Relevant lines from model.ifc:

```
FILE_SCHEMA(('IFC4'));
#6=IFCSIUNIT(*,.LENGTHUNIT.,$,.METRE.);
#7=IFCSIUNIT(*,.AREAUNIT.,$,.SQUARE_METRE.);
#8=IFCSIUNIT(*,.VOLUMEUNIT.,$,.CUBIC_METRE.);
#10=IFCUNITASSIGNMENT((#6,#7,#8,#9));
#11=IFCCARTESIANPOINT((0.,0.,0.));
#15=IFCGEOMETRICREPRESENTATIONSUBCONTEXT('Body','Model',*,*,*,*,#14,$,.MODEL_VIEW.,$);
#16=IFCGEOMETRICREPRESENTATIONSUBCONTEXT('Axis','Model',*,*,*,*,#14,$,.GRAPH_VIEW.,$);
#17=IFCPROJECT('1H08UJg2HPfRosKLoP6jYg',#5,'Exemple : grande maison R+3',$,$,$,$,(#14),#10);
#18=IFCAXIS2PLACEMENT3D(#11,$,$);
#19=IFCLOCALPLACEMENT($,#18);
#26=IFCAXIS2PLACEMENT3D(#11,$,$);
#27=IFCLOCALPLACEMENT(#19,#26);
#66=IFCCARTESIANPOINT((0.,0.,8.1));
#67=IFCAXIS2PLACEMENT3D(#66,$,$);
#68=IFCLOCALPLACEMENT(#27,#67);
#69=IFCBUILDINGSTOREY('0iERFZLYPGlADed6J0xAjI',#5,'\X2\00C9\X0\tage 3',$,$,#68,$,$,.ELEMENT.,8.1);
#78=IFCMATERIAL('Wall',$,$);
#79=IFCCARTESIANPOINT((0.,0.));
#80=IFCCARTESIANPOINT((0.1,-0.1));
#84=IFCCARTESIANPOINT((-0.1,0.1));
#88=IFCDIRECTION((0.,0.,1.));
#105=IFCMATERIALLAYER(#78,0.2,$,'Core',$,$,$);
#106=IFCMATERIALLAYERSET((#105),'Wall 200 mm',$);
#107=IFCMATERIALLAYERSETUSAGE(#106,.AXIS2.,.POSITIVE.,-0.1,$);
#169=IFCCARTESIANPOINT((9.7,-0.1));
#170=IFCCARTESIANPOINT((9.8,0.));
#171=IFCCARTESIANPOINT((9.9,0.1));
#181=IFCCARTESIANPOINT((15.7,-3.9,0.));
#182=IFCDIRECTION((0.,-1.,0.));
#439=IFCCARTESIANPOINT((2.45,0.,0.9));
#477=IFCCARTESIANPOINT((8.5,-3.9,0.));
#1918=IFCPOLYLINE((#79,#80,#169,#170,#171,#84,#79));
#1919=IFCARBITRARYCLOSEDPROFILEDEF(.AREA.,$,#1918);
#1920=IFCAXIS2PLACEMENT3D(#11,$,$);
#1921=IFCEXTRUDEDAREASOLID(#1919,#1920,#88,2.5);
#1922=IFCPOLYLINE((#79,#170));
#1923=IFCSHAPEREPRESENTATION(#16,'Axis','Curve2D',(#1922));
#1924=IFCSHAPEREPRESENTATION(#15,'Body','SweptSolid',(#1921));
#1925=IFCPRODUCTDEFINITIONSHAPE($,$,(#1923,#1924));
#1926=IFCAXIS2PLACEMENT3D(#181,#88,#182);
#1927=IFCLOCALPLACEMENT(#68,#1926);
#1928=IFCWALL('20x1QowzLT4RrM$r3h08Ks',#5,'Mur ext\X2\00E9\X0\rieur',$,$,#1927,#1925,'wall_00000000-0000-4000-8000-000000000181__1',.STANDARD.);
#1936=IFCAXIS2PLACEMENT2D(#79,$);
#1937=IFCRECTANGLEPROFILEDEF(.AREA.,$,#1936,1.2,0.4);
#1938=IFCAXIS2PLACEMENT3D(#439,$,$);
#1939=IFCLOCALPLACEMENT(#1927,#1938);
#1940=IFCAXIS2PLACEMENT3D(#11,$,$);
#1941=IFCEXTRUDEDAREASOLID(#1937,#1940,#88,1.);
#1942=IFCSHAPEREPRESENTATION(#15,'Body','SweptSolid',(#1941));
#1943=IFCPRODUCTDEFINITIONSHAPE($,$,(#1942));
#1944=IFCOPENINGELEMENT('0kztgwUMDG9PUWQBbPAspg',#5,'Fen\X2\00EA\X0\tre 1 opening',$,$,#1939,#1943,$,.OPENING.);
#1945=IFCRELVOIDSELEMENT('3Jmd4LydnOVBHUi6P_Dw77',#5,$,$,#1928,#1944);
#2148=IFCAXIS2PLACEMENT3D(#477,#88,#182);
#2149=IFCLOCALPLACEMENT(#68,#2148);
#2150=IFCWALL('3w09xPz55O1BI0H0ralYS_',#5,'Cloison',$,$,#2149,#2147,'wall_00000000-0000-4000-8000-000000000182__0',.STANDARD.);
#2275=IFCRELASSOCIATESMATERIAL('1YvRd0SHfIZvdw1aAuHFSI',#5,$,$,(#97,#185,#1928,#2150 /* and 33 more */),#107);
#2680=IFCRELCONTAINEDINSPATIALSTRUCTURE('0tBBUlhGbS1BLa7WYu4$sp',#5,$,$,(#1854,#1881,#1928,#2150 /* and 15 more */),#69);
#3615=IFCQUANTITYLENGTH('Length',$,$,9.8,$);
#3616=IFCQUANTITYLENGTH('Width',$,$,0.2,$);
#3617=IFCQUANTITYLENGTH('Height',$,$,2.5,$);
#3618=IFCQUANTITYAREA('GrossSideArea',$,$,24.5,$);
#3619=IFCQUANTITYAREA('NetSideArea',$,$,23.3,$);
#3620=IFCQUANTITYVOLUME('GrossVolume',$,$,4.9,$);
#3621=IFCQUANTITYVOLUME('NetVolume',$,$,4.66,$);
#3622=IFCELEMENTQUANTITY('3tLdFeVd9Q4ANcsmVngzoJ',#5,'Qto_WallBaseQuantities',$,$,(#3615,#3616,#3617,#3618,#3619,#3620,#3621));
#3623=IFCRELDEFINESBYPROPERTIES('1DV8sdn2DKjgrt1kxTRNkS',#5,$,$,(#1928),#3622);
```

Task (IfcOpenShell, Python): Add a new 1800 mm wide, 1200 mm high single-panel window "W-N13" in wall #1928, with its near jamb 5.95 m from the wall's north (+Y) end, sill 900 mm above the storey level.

```python
import numpy as np
import ifcopenshell
import ifcopenshell.api.feature
import ifcopenshell.api.geometry
import ifcopenshell.api.pset
import ifcopenshell.api.root
import ifcopenshell.api.spatial
import ifcopenshell.geom
import ifcopenshell.util.element
import ifcopenshell.util.placement
import ifcopenshell.util.representation
import ifcopenshell.util.shape
import ifcopenshell.util.unit

model = ifcopenshell.open("model.ifc")
unit_scale = ifcopenshell.util.unit.calculate_unit_scale(model)
area_scale = ifcopenshell.util.unit.calculate_unit_scale(model, "AREAUNIT")
volume_scale = ifcopenshell.util.unit.calculate_unit_scale(model, "VOLUMEUNIT")
settings = ifcopenshell.geom.settings()


def volume(element):
    """Net volume in cubic metres, openings subtracted."""
    shape = ifcopenshell.geom.create_shape(settings, element)
    return ifcopenshell.util.shape.get_volume(shape.geometry)


wall = model.by_guid("20x1QowzLT4RrM$r3h08Ks")
storey = ifcopenshell.util.element.get_container(wall, ifc_class="IfcBuildingStorey")
context = ifcopenshell.util.representation.get_context(model, "Model", "Body", "MODEL_VIEW")
before = volume(wall)

width, height, from_end, sill = 1.8, 1.2, 5.95, 0.9  # metres

# The wall runs along its own X axis, and the end named is its -X end.
wall_shape = ifcopenshell.geom.create_shape(settings, wall)
x, y, z = ifcopenshell.util.shape.get_vertices(wall_shape.geometry).T
start = x.min() + from_end
face, thickness = float(y.min()), float(y.max() - y.min())
wall_matrix = ifcopenshell.util.placement.get_local_placement(wall.ObjectPlacement)
level = ifcopenshell.util.placement.get_local_placement(storey.ObjectPlacement)[2, 3]


def in_wall(x, y):
    """Placement at x, y metres in the wall's axes, at sill height."""
    matrix = wall_matrix.copy()
    matrix[:, 3] = wall_matrix @ np.array([x / unit_scale, y / unit_scale, 0.0, 1.0])
    matrix[2, 3] = level + sill / unit_scale
    return matrix


# Opening: a box that overshoots both wall faces by 50 mm.
opening = ifcopenshell.api.root.create_entity(model, ifc_class="IfcOpeningElement", predefined_type="OPENING")
box = ifcopenshell.api.geometry.add_wall_representation(
    model, context=context, length=width, height=height, thickness=thickness + 0.1
)
ifcopenshell.api.geometry.assign_representation(model, product=opening, representation=box)
ifcopenshell.api.geometry.edit_object_placement(model, product=opening, matrix=in_wall(start, face - 0.05), is_si=False)
ifcopenshell.api.feature.add_feature(model, feature=opening, element=wall)

window = ifcopenshell.api.root.create_entity(model, ifc_class="IfcWindow", name="W-N13", predefined_type="WINDOW")
window.OverallWidth, window.OverallHeight = width / unit_scale, height / unit_scale
window.PartitioningType = "SINGLE_PANEL"
body = ifcopenshell.api.geometry.add_window_representation(
    model,
    context=context,
    overall_width=window.OverallWidth,
    overall_height=window.OverallHeight,
    partition_type="SINGLE_PANEL",
)
ifcopenshell.api.geometry.assign_representation(model, product=window, representation=body)
ifcopenshell.api.spatial.assign_container(model, products=[window], relating_structure=storey)
ifcopenshell.api.feature.add_filling(model, opening=opening, element=window)

# Centre the window in the wall's thickness.
ifcopenshell.api.geometry.edit_object_placement(model, product=window, matrix=in_wall(start, face), is_si=False)
window_shape = ifcopenshell.geom.create_shape(settings, window)
depth = ifcopenshell.util.shape.get_vertices(window_shape.geometry)[:, 1]
offset = face + thickness / 2 - (depth.min() + depth.max()) / 2
ifcopenshell.api.geometry.edit_object_placement(model, product=window, matrix=in_wall(start, offset), is_si=False)

after = volume(wall)

# Update the wall's stored quantities.
qto = model.by_id(ifcopenshell.util.element.get_pset(wall, "Qto_WallBaseQuantities", should_inherit=False)["id"])
ifcopenshell.api.pset.edit_qto(model, qto=qto, properties={
    "NetSideArea": after / thickness / area_scale,
    "NetVolume": after / volume_scale,
})

print(f"wall volume {before:.3f} -> {after:.3f} m3")

model.write("model_v2.ifc")
```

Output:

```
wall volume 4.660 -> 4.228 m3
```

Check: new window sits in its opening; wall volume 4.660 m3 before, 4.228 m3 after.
